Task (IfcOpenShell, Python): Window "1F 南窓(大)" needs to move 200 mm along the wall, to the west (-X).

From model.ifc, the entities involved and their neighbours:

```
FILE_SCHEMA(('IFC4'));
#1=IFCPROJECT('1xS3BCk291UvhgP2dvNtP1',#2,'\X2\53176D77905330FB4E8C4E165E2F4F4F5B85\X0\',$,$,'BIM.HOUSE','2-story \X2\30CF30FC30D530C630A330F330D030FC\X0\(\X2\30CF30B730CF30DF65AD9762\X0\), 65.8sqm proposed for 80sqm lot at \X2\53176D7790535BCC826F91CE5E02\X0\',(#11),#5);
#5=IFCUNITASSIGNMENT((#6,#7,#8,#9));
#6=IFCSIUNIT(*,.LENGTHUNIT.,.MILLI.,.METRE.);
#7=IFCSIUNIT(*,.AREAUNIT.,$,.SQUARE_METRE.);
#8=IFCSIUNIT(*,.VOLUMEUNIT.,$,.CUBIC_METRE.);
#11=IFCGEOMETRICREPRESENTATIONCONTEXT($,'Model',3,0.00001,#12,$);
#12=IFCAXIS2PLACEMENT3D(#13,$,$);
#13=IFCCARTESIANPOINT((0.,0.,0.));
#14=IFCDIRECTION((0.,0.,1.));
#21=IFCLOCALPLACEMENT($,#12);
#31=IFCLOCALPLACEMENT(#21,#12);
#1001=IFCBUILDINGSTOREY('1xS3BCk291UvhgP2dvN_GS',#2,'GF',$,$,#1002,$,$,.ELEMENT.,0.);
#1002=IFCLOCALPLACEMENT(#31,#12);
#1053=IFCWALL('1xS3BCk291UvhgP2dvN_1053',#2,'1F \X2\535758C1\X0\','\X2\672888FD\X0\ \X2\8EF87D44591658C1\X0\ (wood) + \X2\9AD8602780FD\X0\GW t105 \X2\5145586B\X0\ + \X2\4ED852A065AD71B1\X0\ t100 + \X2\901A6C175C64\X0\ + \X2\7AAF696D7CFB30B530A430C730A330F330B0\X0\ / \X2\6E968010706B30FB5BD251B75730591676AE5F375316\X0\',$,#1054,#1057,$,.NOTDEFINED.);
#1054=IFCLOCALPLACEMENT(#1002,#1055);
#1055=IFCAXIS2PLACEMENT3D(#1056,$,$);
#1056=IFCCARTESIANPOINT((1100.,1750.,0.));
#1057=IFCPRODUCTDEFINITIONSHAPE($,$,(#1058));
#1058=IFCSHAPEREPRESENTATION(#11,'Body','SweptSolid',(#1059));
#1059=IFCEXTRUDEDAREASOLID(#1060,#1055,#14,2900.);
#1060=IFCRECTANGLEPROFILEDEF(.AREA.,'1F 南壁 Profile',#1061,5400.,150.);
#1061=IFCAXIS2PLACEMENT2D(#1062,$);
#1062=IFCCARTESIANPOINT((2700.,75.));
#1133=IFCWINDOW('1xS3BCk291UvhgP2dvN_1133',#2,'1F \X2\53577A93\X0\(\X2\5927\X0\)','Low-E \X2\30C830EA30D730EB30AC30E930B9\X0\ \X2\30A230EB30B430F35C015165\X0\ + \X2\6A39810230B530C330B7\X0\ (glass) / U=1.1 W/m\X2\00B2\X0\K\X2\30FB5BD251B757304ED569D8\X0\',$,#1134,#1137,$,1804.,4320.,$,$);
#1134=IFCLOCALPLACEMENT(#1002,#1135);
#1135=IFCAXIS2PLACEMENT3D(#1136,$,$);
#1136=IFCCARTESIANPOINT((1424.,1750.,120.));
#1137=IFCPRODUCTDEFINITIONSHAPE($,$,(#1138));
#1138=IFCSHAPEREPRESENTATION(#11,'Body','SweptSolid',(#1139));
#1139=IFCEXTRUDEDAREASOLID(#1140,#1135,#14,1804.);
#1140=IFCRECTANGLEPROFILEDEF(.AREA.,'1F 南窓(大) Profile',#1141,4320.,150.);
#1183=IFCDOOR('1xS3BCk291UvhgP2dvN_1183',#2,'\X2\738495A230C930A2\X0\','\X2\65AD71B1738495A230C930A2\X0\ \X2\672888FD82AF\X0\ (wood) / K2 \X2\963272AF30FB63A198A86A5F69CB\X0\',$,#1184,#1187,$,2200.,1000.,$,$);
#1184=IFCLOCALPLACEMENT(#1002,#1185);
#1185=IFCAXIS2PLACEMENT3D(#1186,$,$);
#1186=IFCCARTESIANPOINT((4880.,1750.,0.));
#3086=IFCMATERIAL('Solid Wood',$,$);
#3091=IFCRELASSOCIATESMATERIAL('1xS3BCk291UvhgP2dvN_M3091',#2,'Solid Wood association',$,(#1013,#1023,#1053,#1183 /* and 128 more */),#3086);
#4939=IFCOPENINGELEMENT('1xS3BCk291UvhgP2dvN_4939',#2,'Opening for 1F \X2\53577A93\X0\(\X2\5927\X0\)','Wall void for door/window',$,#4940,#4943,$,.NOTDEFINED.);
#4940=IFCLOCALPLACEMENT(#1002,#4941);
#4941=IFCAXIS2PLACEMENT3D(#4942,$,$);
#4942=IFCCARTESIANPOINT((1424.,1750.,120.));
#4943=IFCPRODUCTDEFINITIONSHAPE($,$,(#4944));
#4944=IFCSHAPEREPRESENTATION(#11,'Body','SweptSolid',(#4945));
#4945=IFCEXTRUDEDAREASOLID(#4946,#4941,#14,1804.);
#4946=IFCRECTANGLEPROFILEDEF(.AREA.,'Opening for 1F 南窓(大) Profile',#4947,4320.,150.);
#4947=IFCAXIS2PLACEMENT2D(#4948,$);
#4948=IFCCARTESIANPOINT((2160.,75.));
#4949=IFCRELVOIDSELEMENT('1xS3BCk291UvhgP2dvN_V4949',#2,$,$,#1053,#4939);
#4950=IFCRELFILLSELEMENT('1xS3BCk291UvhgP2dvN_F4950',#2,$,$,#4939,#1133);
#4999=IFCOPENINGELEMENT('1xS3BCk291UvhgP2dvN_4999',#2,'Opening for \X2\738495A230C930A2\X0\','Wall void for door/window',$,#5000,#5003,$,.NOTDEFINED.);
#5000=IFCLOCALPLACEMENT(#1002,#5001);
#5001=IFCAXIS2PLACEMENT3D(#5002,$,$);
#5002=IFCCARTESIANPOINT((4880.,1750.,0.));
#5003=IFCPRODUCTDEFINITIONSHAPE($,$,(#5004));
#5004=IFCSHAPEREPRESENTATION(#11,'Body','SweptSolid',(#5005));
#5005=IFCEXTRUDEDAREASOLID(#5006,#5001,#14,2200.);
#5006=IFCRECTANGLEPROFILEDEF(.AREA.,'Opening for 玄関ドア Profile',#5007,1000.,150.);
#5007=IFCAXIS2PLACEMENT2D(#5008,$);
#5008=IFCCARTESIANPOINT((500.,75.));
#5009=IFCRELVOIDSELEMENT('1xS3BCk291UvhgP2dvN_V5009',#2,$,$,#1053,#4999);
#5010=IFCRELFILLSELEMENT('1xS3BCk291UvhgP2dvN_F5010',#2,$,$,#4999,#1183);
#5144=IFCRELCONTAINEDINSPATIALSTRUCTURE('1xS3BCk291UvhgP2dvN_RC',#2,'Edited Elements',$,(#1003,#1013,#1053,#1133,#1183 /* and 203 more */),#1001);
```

```python
import ifcopenshell
import ifcopenshell.api.geometry
import ifcopenshell.util.placement
import ifcopenshell.util.unit

model = ifcopenshell.open("model.ifc")
unit_scale = ifcopenshell.util.unit.calculate_unit_scale(model)

window = model.by_guid("1xS3BCk291UvhgP2dvN_1133")
opening = window.FillsVoids[0].RelatingOpeningElement
wall = opening.VoidsElements[0].RelatingBuildingElement

wall_matrix = ifcopenshell.util.placement.get_local_placement(wall.ObjectPlacement)
shift = wall_matrix[:3, 0] * -0.2 / unit_scale
before = ifcopenshell.util.placement.get_local_placement(window.ObjectPlacement)[:3, 3].copy()

# The window is not placed relative to its opening, so move both.
for product in (opening, window):
    matrix = ifcopenshell.util.placement.get_local_placement(product.ObjectPlacement)
    matrix[:3, 3] += shift
    ifcopenshell.api.geometry.edit_object_placement(model, product=product, matrix=matrix, is_si=False)

after = ifcopenshell.util.placement.get_local_placement(window.ObjectPlacement)[:3, 3]
print("window moved by", (after - before).round(3) + 0.0)

model.write("model-out.ifc")
```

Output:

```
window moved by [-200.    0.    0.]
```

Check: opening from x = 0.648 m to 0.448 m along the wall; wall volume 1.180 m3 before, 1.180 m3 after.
